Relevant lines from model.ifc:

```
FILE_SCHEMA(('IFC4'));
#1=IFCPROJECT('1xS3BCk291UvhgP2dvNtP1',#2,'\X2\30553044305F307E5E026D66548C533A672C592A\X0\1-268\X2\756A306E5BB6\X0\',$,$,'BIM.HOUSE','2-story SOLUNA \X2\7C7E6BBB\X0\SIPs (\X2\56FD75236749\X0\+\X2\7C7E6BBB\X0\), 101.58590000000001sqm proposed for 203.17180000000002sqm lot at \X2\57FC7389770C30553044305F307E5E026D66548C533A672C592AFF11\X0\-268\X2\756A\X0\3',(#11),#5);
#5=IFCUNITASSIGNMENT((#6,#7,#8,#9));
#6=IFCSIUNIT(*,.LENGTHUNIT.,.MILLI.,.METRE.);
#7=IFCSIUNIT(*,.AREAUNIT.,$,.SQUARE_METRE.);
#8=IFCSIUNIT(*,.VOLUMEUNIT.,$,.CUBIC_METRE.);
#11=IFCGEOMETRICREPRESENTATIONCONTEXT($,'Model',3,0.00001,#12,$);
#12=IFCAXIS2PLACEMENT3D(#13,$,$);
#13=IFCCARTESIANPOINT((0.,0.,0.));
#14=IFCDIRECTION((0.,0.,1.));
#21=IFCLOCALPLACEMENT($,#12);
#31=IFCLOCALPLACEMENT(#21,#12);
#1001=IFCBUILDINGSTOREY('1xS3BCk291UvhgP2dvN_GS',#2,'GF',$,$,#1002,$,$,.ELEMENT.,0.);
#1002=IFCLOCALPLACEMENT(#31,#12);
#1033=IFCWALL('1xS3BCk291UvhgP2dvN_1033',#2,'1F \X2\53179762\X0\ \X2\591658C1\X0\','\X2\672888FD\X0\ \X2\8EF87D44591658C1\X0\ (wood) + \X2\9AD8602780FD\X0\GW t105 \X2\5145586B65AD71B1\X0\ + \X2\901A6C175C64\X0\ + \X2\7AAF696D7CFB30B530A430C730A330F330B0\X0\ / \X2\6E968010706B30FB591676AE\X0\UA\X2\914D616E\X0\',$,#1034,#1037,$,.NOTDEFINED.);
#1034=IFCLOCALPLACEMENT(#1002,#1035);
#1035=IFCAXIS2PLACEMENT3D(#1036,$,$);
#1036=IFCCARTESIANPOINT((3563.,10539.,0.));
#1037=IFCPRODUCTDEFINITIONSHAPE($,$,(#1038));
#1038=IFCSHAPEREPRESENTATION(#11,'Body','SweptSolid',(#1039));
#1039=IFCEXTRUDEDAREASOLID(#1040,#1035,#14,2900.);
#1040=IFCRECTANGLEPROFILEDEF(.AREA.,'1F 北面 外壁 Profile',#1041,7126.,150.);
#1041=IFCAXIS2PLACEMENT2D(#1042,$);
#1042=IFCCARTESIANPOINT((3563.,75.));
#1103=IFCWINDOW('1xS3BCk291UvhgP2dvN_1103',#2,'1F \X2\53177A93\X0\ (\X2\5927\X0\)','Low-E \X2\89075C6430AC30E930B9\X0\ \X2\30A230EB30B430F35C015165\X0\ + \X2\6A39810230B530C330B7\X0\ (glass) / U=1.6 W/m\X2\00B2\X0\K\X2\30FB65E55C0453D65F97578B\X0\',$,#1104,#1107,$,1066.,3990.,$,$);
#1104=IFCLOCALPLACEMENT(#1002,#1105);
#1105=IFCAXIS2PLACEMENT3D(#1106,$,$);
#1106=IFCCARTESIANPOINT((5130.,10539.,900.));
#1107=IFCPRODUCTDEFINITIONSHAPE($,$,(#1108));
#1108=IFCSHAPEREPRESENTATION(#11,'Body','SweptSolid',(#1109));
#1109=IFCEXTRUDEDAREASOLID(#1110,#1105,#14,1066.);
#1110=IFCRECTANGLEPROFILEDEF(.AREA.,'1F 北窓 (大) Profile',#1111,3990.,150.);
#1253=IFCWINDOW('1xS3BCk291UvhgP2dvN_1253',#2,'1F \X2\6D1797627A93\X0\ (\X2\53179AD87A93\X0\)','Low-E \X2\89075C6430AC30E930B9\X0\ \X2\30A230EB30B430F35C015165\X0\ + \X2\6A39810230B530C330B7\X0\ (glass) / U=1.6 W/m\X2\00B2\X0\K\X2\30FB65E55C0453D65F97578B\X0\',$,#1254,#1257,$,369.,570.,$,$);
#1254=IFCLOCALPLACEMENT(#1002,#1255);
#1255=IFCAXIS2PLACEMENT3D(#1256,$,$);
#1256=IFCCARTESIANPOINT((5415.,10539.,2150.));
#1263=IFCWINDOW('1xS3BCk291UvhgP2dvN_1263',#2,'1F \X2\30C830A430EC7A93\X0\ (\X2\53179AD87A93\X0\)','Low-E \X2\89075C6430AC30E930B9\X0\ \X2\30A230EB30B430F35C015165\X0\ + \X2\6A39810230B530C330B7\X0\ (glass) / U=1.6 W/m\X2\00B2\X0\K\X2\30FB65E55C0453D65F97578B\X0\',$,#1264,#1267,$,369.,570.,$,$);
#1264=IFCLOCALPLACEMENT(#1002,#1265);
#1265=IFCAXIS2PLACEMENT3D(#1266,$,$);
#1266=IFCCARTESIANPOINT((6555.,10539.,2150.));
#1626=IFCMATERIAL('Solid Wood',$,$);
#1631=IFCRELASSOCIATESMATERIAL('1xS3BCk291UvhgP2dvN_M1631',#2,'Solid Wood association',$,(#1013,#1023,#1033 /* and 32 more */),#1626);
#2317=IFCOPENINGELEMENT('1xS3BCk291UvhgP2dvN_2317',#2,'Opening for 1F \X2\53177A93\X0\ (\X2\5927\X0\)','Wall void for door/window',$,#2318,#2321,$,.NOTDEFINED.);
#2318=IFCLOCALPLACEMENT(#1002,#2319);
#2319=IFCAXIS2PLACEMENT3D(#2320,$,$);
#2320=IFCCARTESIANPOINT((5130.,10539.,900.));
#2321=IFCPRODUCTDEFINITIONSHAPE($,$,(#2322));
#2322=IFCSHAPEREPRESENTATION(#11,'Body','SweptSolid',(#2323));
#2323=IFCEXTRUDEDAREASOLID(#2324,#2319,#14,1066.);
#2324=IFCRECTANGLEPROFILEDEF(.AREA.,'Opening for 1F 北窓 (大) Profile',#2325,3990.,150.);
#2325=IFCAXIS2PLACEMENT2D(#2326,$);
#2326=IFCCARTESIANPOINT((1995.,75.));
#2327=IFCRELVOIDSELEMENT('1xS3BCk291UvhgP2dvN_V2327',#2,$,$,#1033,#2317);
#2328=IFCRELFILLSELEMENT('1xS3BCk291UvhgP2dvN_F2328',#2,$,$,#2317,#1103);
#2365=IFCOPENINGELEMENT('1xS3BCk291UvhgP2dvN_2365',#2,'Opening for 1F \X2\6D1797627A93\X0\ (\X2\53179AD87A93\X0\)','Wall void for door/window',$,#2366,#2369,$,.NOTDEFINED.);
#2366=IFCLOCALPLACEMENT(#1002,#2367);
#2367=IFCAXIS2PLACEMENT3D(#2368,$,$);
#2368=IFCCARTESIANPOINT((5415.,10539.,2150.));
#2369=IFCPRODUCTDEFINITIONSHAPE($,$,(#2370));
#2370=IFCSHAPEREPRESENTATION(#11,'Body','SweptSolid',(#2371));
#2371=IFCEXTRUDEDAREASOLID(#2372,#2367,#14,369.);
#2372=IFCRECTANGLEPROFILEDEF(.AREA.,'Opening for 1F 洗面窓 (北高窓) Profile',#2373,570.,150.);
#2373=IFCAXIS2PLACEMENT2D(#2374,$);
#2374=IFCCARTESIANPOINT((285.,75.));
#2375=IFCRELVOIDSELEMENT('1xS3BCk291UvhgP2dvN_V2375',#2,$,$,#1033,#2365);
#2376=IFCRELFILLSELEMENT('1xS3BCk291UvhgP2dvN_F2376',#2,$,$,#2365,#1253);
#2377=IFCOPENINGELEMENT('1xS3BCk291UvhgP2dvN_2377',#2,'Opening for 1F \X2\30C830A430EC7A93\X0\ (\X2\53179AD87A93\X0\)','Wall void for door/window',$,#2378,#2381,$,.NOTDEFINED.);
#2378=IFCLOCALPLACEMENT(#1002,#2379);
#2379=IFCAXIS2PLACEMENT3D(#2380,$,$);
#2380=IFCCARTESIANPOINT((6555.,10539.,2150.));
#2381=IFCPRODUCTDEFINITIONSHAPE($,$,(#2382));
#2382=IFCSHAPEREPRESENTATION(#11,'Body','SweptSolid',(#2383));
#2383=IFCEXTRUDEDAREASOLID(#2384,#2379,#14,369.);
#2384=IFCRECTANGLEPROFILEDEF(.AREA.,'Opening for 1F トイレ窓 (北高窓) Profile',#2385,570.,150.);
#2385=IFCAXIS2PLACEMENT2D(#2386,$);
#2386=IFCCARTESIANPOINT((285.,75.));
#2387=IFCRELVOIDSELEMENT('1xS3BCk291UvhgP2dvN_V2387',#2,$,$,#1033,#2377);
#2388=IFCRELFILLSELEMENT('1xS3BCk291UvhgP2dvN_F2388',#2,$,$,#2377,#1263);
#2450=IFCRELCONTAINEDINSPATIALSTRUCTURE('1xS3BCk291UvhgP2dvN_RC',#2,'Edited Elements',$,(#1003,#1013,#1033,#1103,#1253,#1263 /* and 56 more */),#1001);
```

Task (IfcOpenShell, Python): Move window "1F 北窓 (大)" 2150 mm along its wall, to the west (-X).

```python
import ifcopenshell
import ifcopenshell.api.geometry
import ifcopenshell.util.placement
import ifcopenshell.util.unit

model = ifcopenshell.open("model.ifc")
unit_scale = ifcopenshell.util.unit.calculate_unit_scale(model)

window = model.by_guid("1xS3BCk291UvhgP2dvN_1103")
opening = window.FillsVoids[0].RelatingOpeningElement
wall = opening.VoidsElements[0].RelatingBuildingElement

wall_matrix = ifcopenshell.util.placement.get_local_placement(wall.ObjectPlacement)
shift = wall_matrix[:3, 0] * -2.15 / unit_scale
before = ifcopenshell.util.placement.get_local_placement(window.ObjectPlacement)[:3, 3].copy()

# The window is not placed relative to its opening, so move both.
for product in (opening, window):
    matrix = ifcopenshell.util.placement.get_local_placement(product.ObjectPlacement)
    matrix[:3, 3] += shift
    ifcopenshell.api.geometry.edit_object_placement(model, product=product, matrix=matrix, is_si=False)

after = ifcopenshell.util.placement.get_local_placement(window.ObjectPlacement)[:3, 3]
print("window moved by", (after - before).round(3) + 0.0)

model.write("model_updated.ifc")
```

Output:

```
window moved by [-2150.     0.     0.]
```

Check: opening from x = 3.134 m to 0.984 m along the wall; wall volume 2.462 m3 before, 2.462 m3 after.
